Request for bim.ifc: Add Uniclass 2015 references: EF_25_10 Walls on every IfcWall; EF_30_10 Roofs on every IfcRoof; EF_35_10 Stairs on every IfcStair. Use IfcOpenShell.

First a look at what the model holds.

```python
import ifcopenshell

model = ifcopenshell.open("bim.ifc")
print(model.schema)
print("classifications:", [c.Name for c in model.by_type("IfcClassification")])
for ifc_class in ("IfcDoor", "IfcRoof", "IfcStair", "IfcWall", "IfcWindow"):
    print(ifc_class, len(model.by_type(ifc_class)))
```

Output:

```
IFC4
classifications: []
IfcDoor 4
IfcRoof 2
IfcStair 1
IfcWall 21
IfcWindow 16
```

```python
import ifcopenshell
import ifcopenshell.api.classification

model = ifcopenshell.open("bim.ifc")

system = ifcopenshell.api.classification.add_classification(model, classification="Uniclass 2015")

codes = {
    "IfcWall": ("EF_25_10", "Walls"),
    "IfcRoof": ("EF_30_10", "Roofs"),
    "IfcStair": ("EF_35_10", "Stairs"),
}
for ifc_class, (code, name) in codes.items():
    products = model.by_type(ifc_class)
    ifcopenshell.api.classification.add_reference(
        model, products=products, classification=system, identification=code, name=name
    )
    print(code, len(products))

model.write("bim-out.ifc")
```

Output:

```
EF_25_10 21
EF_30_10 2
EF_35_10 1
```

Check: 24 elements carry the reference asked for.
